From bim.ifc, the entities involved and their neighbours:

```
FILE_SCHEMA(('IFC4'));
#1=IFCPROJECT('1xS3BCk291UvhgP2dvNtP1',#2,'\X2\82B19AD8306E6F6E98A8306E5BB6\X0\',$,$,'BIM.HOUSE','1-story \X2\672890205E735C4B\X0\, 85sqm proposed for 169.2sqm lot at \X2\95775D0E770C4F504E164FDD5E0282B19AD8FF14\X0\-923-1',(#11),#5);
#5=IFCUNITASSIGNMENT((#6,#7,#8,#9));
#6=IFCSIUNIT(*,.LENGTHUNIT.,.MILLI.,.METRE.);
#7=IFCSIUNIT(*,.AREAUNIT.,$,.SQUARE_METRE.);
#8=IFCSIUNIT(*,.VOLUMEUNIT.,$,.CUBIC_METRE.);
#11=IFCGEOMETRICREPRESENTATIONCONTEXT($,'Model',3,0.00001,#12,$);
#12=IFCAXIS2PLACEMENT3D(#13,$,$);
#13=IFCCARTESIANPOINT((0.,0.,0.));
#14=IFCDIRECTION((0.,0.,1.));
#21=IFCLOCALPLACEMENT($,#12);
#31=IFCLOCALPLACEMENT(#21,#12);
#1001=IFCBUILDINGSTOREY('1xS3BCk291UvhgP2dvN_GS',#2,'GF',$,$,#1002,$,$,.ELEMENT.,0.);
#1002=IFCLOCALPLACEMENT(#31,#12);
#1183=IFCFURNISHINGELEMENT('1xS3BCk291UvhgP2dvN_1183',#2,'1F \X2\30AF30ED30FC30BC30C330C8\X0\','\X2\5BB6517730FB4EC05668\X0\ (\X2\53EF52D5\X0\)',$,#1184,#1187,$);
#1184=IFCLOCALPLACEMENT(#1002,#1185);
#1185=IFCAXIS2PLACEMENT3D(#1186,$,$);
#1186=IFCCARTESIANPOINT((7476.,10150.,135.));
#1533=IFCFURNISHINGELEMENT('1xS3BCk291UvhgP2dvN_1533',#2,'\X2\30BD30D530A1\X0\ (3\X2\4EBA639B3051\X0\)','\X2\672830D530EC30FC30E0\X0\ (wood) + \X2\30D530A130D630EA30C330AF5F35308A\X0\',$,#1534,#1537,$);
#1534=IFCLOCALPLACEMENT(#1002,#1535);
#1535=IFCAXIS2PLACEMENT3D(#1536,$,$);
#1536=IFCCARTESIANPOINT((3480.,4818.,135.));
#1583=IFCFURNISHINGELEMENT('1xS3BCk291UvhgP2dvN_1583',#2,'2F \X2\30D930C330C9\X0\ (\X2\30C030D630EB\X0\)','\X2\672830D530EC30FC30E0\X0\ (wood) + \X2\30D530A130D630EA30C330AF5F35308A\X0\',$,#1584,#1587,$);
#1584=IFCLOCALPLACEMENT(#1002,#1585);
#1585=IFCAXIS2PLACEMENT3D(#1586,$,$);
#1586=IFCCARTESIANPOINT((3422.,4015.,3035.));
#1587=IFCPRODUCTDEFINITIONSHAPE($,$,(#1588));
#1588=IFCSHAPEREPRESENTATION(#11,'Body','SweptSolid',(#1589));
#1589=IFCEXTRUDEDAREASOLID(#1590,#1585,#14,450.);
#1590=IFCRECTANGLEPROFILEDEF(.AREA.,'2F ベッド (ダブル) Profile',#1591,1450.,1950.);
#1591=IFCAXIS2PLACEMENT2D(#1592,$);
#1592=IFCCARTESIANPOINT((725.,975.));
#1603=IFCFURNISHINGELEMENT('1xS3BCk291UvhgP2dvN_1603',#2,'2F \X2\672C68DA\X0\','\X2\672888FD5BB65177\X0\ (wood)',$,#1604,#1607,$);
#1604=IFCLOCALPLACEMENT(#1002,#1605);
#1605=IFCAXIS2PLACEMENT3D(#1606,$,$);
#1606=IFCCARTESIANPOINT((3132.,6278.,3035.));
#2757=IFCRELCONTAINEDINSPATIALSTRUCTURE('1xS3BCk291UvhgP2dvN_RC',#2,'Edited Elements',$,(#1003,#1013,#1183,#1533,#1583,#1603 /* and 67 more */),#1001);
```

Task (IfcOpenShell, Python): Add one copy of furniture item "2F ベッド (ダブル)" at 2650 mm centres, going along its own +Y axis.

```python
import ifcopenshell
import ifcopenshell.api.geometry
import ifcopenshell.api.root
import ifcopenshell.util.element
import ifcopenshell.util.placement
import ifcopenshell.util.unit

model = ifcopenshell.open("bim.ifc")
unit_scale = ifcopenshell.util.unit.calculate_unit_scale(model)


def reuse_history(source, copy):
    """copy_class also copies each property set's owner history, people and application; keep the originals."""
    for rel in copy.IsDefinedBy:
        if rel.is_a("IfcRelDefinesByProperties") and (history := rel.RelatingPropertyDefinition.OwnerHistory):
            rel.RelatingPropertyDefinition.OwnerHistory = source.OwnerHistory
            ifcopenshell.util.element.remove_deep2(model, history)


source = model.by_guid("1xS3BCk291UvhgP2dvN_1583")
base = ifcopenshell.util.placement.get_local_placement(source.ObjectPlacement)
step = base[:3, 1] * 2.65 / unit_scale

for i in range(1, 2):
    copy = ifcopenshell.api.root.copy_class(model, product=source)
    copy.Representation = ifcopenshell.util.element.copy_deep(
        model, source.Representation, exclude=["IfcGeometricRepresentationContext", "IfcRepresentationMap"]
    )
    reuse_history(source, copy)
    matrix = base.copy()
    matrix[:3, 3] += i * step
    print("added at", matrix[:3, 3].round(3) + 0.0)
    ifcopenshell.api.geometry.edit_object_placement(model, product=copy, matrix=matrix, is_si=False)

model.write("bim_updated.ifc")
```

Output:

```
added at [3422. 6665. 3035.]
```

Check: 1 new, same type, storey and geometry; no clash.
